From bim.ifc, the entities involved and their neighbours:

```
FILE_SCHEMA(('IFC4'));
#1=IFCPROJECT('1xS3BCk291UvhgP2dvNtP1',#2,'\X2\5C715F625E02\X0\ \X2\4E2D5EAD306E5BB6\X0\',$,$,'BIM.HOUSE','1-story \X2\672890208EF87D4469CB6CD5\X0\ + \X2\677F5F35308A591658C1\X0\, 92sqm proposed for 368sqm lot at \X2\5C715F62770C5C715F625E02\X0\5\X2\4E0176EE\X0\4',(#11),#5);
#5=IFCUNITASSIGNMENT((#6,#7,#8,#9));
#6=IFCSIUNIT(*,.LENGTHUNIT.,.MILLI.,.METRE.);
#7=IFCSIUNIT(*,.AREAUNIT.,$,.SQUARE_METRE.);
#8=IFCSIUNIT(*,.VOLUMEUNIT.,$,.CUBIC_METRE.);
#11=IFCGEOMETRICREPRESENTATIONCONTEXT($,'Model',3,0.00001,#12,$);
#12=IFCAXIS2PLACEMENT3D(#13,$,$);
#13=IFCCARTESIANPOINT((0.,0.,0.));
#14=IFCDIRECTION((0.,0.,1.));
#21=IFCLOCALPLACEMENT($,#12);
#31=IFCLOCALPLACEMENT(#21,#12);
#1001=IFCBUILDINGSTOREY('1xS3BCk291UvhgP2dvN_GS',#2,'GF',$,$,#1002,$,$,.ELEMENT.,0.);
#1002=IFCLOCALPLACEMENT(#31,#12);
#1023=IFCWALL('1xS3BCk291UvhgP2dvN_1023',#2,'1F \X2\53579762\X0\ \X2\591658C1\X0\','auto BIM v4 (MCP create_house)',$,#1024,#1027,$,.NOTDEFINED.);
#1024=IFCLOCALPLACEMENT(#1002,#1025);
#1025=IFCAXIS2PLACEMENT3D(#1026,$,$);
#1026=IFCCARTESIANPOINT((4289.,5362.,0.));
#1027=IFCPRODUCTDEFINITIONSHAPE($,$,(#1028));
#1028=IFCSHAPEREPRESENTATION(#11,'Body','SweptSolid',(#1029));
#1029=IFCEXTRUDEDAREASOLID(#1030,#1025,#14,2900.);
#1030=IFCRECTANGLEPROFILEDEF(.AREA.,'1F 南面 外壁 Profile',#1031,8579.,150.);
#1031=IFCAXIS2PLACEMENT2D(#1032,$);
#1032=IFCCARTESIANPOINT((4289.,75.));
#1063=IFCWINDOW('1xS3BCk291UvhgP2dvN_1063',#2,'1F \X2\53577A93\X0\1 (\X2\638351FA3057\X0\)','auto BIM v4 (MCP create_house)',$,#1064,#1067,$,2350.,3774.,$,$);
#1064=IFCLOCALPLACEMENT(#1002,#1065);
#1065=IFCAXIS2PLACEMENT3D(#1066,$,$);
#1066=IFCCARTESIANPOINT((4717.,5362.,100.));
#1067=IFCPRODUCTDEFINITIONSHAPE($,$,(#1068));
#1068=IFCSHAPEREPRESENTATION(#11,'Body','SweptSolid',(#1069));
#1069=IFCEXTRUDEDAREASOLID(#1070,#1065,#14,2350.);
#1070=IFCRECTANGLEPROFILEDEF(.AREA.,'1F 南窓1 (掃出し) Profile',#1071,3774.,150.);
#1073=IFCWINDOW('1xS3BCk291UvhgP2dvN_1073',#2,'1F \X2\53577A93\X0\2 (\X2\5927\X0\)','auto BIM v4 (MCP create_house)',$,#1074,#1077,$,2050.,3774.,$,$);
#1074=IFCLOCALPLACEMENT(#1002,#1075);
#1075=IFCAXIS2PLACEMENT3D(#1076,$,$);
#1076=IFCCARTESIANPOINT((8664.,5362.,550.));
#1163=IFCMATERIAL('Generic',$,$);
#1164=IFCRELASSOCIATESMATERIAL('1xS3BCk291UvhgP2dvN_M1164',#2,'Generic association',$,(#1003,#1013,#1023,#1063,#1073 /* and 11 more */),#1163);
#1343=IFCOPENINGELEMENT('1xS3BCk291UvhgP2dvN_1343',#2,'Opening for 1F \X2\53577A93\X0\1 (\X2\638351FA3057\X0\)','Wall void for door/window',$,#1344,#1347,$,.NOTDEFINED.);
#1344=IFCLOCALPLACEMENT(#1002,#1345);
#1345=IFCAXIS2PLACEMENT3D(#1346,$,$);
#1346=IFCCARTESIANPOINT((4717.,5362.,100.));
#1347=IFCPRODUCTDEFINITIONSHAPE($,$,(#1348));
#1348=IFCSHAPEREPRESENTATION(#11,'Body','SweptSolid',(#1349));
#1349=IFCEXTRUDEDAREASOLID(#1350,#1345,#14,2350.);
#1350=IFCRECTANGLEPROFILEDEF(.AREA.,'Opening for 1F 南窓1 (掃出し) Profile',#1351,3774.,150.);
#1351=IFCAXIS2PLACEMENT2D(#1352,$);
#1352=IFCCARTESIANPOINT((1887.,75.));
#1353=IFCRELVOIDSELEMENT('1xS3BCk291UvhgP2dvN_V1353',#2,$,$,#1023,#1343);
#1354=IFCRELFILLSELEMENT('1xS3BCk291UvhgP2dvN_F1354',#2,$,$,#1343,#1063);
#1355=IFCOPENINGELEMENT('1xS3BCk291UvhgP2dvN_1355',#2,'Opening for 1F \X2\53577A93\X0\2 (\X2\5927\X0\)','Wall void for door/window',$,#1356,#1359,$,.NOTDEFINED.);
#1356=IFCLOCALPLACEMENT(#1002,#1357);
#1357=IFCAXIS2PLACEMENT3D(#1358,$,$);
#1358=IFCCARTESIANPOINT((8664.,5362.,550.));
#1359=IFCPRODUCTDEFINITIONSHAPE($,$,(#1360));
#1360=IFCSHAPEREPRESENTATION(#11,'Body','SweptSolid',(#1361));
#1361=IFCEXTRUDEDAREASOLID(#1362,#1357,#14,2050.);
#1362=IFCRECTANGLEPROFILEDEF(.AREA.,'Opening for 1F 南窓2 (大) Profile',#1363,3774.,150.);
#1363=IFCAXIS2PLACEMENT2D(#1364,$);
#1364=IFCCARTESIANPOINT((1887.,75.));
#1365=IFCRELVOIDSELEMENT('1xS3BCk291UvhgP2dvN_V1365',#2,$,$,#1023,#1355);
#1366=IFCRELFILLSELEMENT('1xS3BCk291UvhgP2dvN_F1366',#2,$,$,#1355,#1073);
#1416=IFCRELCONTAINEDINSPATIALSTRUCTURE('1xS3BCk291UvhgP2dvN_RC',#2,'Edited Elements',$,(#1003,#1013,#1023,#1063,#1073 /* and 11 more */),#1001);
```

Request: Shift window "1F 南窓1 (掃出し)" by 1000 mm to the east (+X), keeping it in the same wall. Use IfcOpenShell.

```python
import ifcopenshell
import ifcopenshell.api.geometry
import ifcopenshell.util.placement
import ifcopenshell.util.unit

model = ifcopenshell.open("bim.ifc")
unit_scale = ifcopenshell.util.unit.calculate_unit_scale(model)

window = model.by_id(1063)
opening = window.FillsVoids[0].RelatingOpeningElement
wall = opening.VoidsElements[0].RelatingBuildingElement

wall_matrix = ifcopenshell.util.placement.get_local_placement(wall.ObjectPlacement)
shift = wall_matrix[:3, 0] * 1 / unit_scale
before = ifcopenshell.util.placement.get_local_placement(window.ObjectPlacement)[:3, 3].copy()

# The window is not placed relative to its opening, so move both.
for product in (opening, window):
    matrix = ifcopenshell.util.placement.get_local_placement(product.ObjectPlacement)
    matrix[:3, 3] += shift
    ifcopenshell.api.geometry.edit_object_placement(model, product=product, matrix=matrix, is_si=False)

after = ifcopenshell.util.placement.get_local_placement(window.ObjectPlacement)[:3, 3]
print("window moved by", (after - before).round(3) + 0.0)

model.write("bim_updated.ifc")
```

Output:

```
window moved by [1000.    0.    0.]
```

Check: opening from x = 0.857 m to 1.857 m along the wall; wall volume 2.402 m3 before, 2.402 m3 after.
